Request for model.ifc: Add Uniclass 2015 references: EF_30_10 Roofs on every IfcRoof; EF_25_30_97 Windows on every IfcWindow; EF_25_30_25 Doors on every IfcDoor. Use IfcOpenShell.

First a look at what the model holds.

```python
import ifcopenshell

model = ifcopenshell.open("model.ifc")
print(model.schema)
print("classifications:", [c.Name for c in model.by_type("IfcClassification")])
for ifc_class in ("IfcDoor", "IfcRoof", "IfcStair", "IfcWall", "IfcWindow"):
    print(ifc_class, len(model.by_type(ifc_class)))
```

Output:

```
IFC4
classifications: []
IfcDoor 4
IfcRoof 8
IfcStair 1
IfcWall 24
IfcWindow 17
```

```python
import ifcopenshell
import ifcopenshell.api.classification

model = ifcopenshell.open("model.ifc")

system = ifcopenshell.api.classification.add_classification(model, classification="Uniclass 2015")

codes = {
    "IfcRoof": ("EF_30_10", "Roofs"),
    "IfcWindow": ("EF_25_30_97", "Windows"),
    "IfcDoor": ("EF_25_30_25", "Doors"),
}
for ifc_class, (code, name) in codes.items():
    products = model.by_type(ifc_class)
    ifcopenshell.api.classification.add_reference(
        model, products=products, classification=system, identification=code, name=name
    )
    print(code, len(products))

model.write("model-out.ifc")
```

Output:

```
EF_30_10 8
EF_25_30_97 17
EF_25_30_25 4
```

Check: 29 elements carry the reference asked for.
